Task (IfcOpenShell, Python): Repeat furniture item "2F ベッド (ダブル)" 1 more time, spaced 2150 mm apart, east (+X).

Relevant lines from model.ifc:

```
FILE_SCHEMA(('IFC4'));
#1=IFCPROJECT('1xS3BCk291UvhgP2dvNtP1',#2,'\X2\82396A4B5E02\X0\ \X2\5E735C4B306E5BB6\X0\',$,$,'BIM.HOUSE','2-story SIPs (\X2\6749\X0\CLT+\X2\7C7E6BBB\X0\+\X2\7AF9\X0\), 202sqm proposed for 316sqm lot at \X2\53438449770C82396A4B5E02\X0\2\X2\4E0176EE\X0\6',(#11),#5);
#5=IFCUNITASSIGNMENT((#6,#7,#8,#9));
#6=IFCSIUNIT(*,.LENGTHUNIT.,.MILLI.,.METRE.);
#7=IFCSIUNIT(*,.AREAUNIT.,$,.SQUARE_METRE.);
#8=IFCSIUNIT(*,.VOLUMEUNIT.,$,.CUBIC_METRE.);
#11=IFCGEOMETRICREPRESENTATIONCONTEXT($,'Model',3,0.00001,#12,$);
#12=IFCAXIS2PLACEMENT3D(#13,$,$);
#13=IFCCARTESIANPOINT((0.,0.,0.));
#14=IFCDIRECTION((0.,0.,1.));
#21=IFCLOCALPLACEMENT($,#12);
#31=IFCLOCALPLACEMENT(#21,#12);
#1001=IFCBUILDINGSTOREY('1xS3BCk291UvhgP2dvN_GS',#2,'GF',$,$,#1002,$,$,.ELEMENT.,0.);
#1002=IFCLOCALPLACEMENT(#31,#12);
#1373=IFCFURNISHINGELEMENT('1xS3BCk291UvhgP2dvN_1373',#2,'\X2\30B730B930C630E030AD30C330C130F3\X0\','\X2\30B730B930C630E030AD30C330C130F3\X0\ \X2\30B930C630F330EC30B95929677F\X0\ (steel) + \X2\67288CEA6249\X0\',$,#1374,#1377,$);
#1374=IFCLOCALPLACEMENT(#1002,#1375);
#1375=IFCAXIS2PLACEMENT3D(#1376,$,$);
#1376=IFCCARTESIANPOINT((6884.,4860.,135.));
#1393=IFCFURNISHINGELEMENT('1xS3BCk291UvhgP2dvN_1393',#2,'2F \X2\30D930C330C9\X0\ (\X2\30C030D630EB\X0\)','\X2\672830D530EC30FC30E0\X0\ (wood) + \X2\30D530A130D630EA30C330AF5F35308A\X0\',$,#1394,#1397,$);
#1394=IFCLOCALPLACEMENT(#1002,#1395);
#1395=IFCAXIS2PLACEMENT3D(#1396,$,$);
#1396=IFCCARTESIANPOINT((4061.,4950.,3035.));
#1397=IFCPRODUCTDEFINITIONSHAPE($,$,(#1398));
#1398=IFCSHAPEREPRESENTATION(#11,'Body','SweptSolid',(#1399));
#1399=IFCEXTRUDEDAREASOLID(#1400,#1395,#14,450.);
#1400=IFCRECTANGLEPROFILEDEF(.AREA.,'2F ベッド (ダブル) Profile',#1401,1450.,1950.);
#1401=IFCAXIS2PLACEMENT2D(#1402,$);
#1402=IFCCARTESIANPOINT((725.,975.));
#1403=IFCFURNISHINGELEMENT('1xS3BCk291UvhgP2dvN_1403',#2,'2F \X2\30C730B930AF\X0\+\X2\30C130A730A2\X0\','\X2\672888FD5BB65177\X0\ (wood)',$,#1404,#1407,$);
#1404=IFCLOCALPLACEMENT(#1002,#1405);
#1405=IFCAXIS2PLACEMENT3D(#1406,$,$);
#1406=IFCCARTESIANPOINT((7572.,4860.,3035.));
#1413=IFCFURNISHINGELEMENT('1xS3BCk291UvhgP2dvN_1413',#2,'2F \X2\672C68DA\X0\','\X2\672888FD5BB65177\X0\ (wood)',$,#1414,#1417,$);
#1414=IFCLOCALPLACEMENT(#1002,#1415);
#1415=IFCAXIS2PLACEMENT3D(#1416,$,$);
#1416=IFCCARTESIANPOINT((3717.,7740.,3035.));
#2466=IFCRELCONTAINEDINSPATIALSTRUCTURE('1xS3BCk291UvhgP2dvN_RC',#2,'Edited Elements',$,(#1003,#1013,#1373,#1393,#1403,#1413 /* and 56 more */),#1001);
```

```python
import numpy as np
import ifcopenshell
import ifcopenshell.api.geometry
import ifcopenshell.api.root
import ifcopenshell.util.element
import ifcopenshell.util.placement

model = ifcopenshell.open("model.ifc")


def reuse_history(source, copy):
    """copy_class also copies each property set's owner history, people and application; keep the originals."""
    for rel in copy.IsDefinedBy:
        if rel.is_a("IfcRelDefinesByProperties") and (history := rel.RelatingPropertyDefinition.OwnerHistory):
            rel.RelatingPropertyDefinition.OwnerHistory = source.OwnerHistory
            ifcopenshell.util.element.remove_deep2(model, history)


source = model.by_guid("1xS3BCk291UvhgP2dvN_1393")
base = ifcopenshell.util.placement.get_local_placement(source.ObjectPlacement)
step = np.array([1.0, 0.0, 0.0]) * 2150.0

for i in range(1, 2):
    copy = ifcopenshell.api.root.copy_class(model, product=source)
    copy.Representation = ifcopenshell.util.element.copy_deep(
        model, source.Representation, exclude=["IfcGeometricRepresentationContext", "IfcRepresentationMap"]
    )
    reuse_history(source, copy)
    matrix = base.copy()
    matrix[:3, 3] += i * step
    print("added at", matrix[:3, 3].round(3) + 0.0)
    ifcopenshell.api.geometry.edit_object_placement(model, product=copy, matrix=matrix, is_si=False)

model.write("model_v2.ifc")
```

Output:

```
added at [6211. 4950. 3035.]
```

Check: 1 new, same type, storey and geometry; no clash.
